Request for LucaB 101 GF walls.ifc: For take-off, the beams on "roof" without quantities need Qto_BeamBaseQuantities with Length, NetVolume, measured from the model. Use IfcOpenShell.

First a look at what the model holds.

```python
import ifcopenshell
import ifcopenshell.util.element
import ifcopenshell.util.unit

model = ifcopenshell.open("LucaB 101 GF walls.ifc")
print(model.schema)
for unit_type in ("LENGTHUNIT", "AREAUNIT", "VOLUMEUNIT"):
    print(unit_type, ifcopenshell.util.unit.calculate_unit_scale(model, unit_type))
storey = next(s for s in model.by_type("IfcBuildingStorey") if s.Name == "roof")
beams = [e for e in ifcopenshell.util.element.get_decomposition(storey) if e.is_a("IfcBeam")]
for e in sorted(beams, key=lambda e: e.id()):
    print(e.id(), e.is_a(), e.Name, list(ifcopenshell.util.element.get_psets(e, qtos_only=True)), sep=" | ")
```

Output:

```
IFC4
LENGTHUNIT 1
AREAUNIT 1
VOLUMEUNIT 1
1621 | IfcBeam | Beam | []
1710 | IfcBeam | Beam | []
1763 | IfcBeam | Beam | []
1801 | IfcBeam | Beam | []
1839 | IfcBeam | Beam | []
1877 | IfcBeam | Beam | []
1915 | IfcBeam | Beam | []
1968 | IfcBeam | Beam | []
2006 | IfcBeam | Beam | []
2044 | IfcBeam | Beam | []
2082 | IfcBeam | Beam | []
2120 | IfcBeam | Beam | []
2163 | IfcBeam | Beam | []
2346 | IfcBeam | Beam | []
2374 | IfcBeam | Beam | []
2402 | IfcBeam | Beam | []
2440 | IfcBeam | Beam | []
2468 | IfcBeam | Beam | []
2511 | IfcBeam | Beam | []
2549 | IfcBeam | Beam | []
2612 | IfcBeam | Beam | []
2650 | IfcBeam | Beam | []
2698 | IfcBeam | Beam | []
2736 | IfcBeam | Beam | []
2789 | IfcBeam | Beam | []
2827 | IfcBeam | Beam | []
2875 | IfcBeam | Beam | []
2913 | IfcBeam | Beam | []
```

```python
import ifcopenshell
import ifcopenshell.api.pset
import ifcopenshell.geom
import ifcopenshell.util.element
import ifcopenshell.util.shape
import ifcopenshell.util.unit

model = ifcopenshell.open("LucaB 101 GF walls.ifc")
unit_scale = ifcopenshell.util.unit.calculate_unit_scale(model)
volume_scale = ifcopenshell.util.unit.calculate_unit_scale(model, "VOLUMEUNIT")
settings = ifcopenshell.geom.settings()

storey = next(s for s in model.by_type("IfcBuildingStorey") if s.Name == "roof")
beams = [e for e in ifcopenshell.util.element.get_decomposition(storey) if e.is_a("IfcBeam")]

for e in sorted(beams, key=lambda e: e.id()):
    if ifcopenshell.util.element.get_psets(e, qtos_only=True, should_inherit=False):
        continue
    # Geometry comes back in metres, in the element's own axes.
    shape = ifcopenshell.geom.create_shape(settings, e)
    values = {
        "Length": ifcopenshell.util.shape.get_max_xyz(shape.geometry) / unit_scale,
        "NetVolume": ifcopenshell.util.shape.get_volume(shape.geometry) / volume_scale,
    }
    qto = ifcopenshell.api.pset.add_qto(model, product=e, name="Qto_BeamBaseQuantities")
    ifcopenshell.api.pset.edit_qto(model, qto=qto, properties=values)
    print(e.id(), {k: round(v, 3) for k, v in values.items()})

model.write("LucaB 101 GF walls_rev.ifc")
```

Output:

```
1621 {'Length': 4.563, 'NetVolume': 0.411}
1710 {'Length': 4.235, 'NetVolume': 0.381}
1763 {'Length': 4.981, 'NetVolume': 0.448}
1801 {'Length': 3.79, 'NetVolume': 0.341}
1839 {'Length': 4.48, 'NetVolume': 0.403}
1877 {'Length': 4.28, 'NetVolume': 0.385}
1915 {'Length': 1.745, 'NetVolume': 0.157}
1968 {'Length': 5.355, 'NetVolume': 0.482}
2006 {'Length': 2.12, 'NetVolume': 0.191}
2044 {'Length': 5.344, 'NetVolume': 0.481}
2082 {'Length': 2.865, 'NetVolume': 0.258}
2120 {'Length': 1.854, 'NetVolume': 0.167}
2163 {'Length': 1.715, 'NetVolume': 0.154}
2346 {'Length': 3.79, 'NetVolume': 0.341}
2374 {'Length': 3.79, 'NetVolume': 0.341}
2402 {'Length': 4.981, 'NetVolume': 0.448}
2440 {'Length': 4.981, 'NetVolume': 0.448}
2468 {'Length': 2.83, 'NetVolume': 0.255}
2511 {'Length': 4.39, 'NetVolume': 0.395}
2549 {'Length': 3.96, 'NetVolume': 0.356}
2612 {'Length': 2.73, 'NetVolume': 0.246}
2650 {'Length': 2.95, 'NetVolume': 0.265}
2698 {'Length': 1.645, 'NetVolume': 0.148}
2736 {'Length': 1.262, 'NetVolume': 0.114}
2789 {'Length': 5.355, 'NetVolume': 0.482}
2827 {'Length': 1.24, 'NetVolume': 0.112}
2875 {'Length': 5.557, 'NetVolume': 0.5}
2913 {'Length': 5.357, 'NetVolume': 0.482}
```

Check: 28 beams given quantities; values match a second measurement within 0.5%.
